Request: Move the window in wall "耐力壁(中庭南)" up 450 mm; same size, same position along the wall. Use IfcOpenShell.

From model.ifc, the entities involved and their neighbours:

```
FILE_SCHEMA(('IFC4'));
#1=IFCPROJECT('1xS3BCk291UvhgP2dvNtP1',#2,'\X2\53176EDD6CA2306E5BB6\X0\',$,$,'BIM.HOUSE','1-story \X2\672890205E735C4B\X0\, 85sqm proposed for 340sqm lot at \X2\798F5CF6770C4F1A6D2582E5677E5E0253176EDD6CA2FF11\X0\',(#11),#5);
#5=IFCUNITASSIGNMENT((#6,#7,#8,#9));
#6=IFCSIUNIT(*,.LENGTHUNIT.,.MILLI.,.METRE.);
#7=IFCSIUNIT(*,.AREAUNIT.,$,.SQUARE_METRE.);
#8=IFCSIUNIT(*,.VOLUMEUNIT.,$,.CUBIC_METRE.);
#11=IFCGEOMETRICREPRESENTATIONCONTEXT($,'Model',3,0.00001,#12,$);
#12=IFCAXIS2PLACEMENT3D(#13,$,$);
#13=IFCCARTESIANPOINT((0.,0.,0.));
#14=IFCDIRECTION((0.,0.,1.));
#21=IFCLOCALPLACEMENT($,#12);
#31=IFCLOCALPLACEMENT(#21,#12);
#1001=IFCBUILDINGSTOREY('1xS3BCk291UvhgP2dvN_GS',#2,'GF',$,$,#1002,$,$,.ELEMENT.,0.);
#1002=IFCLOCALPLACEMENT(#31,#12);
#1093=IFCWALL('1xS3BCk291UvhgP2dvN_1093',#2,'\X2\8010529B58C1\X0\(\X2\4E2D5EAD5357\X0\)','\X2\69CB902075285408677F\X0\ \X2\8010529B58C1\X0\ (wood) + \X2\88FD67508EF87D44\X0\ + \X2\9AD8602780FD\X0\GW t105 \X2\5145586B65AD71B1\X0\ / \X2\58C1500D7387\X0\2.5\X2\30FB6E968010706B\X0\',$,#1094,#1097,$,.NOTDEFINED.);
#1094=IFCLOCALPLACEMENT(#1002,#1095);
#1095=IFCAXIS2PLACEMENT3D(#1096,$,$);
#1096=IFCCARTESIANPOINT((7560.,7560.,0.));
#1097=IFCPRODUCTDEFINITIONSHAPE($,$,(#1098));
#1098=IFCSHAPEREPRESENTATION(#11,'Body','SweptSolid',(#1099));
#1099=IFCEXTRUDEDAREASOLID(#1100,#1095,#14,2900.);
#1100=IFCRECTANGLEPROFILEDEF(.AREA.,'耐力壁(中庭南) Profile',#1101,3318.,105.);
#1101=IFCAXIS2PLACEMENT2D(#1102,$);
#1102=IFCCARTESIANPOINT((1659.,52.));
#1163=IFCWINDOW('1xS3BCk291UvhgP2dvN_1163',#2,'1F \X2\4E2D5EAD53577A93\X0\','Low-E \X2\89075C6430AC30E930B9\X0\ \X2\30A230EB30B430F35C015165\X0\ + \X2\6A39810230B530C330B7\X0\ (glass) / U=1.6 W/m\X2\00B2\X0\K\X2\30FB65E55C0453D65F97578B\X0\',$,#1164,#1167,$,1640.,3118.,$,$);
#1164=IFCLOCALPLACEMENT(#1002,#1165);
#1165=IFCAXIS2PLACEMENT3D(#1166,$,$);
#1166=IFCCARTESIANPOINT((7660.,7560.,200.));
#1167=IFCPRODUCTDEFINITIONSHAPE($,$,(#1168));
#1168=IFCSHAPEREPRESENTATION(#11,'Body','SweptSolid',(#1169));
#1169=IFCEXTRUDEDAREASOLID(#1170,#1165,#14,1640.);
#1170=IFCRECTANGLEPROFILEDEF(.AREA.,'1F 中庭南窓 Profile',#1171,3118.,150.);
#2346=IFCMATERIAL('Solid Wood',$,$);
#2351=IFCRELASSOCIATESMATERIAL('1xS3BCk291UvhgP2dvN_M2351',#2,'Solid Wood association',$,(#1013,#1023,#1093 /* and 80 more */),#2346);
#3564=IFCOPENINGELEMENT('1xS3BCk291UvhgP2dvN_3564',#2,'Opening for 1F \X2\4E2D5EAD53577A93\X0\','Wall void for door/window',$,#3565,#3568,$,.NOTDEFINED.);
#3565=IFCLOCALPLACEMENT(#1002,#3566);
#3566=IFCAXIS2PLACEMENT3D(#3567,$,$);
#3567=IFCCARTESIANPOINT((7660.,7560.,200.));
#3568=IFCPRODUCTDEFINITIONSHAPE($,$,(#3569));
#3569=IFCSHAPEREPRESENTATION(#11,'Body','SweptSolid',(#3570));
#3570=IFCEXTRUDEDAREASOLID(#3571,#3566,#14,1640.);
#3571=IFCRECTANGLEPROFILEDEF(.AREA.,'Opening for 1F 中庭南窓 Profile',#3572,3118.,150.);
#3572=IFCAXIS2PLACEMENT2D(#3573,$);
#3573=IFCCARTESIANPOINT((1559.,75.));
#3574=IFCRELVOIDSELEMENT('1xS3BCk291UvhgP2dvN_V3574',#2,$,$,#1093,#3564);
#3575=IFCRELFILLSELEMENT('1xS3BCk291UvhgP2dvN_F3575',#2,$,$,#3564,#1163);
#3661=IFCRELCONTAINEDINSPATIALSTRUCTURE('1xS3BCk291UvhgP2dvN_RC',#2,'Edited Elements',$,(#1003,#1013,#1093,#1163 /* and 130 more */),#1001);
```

```python
import numpy as np
import ifcopenshell
import ifcopenshell.api.geometry
import ifcopenshell.util.placement
import ifcopenshell.util.unit

model = ifcopenshell.open("model.ifc")
unit_scale = ifcopenshell.util.unit.calculate_unit_scale(model)

window = model.by_guid("1xS3BCk291UvhgP2dvN_1163")
opening = window.FillsVoids[0].RelatingOpeningElement
dz = 450.0

shift = np.array([0.0, 0.0, dz])
# The window is not placed relative to its opening, so move both.
for product in (opening, window):
    matrix = ifcopenshell.util.placement.get_local_placement(product.ObjectPlacement)
    matrix[:3, 3] += shift
    ifcopenshell.api.geometry.edit_object_placement(model, product=product, matrix=matrix, is_si=False)

print(f"moved by {dz * unit_scale:+.3f} m")

model.write("model_rev.ifc")
```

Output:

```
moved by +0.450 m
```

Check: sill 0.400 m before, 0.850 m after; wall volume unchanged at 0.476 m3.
